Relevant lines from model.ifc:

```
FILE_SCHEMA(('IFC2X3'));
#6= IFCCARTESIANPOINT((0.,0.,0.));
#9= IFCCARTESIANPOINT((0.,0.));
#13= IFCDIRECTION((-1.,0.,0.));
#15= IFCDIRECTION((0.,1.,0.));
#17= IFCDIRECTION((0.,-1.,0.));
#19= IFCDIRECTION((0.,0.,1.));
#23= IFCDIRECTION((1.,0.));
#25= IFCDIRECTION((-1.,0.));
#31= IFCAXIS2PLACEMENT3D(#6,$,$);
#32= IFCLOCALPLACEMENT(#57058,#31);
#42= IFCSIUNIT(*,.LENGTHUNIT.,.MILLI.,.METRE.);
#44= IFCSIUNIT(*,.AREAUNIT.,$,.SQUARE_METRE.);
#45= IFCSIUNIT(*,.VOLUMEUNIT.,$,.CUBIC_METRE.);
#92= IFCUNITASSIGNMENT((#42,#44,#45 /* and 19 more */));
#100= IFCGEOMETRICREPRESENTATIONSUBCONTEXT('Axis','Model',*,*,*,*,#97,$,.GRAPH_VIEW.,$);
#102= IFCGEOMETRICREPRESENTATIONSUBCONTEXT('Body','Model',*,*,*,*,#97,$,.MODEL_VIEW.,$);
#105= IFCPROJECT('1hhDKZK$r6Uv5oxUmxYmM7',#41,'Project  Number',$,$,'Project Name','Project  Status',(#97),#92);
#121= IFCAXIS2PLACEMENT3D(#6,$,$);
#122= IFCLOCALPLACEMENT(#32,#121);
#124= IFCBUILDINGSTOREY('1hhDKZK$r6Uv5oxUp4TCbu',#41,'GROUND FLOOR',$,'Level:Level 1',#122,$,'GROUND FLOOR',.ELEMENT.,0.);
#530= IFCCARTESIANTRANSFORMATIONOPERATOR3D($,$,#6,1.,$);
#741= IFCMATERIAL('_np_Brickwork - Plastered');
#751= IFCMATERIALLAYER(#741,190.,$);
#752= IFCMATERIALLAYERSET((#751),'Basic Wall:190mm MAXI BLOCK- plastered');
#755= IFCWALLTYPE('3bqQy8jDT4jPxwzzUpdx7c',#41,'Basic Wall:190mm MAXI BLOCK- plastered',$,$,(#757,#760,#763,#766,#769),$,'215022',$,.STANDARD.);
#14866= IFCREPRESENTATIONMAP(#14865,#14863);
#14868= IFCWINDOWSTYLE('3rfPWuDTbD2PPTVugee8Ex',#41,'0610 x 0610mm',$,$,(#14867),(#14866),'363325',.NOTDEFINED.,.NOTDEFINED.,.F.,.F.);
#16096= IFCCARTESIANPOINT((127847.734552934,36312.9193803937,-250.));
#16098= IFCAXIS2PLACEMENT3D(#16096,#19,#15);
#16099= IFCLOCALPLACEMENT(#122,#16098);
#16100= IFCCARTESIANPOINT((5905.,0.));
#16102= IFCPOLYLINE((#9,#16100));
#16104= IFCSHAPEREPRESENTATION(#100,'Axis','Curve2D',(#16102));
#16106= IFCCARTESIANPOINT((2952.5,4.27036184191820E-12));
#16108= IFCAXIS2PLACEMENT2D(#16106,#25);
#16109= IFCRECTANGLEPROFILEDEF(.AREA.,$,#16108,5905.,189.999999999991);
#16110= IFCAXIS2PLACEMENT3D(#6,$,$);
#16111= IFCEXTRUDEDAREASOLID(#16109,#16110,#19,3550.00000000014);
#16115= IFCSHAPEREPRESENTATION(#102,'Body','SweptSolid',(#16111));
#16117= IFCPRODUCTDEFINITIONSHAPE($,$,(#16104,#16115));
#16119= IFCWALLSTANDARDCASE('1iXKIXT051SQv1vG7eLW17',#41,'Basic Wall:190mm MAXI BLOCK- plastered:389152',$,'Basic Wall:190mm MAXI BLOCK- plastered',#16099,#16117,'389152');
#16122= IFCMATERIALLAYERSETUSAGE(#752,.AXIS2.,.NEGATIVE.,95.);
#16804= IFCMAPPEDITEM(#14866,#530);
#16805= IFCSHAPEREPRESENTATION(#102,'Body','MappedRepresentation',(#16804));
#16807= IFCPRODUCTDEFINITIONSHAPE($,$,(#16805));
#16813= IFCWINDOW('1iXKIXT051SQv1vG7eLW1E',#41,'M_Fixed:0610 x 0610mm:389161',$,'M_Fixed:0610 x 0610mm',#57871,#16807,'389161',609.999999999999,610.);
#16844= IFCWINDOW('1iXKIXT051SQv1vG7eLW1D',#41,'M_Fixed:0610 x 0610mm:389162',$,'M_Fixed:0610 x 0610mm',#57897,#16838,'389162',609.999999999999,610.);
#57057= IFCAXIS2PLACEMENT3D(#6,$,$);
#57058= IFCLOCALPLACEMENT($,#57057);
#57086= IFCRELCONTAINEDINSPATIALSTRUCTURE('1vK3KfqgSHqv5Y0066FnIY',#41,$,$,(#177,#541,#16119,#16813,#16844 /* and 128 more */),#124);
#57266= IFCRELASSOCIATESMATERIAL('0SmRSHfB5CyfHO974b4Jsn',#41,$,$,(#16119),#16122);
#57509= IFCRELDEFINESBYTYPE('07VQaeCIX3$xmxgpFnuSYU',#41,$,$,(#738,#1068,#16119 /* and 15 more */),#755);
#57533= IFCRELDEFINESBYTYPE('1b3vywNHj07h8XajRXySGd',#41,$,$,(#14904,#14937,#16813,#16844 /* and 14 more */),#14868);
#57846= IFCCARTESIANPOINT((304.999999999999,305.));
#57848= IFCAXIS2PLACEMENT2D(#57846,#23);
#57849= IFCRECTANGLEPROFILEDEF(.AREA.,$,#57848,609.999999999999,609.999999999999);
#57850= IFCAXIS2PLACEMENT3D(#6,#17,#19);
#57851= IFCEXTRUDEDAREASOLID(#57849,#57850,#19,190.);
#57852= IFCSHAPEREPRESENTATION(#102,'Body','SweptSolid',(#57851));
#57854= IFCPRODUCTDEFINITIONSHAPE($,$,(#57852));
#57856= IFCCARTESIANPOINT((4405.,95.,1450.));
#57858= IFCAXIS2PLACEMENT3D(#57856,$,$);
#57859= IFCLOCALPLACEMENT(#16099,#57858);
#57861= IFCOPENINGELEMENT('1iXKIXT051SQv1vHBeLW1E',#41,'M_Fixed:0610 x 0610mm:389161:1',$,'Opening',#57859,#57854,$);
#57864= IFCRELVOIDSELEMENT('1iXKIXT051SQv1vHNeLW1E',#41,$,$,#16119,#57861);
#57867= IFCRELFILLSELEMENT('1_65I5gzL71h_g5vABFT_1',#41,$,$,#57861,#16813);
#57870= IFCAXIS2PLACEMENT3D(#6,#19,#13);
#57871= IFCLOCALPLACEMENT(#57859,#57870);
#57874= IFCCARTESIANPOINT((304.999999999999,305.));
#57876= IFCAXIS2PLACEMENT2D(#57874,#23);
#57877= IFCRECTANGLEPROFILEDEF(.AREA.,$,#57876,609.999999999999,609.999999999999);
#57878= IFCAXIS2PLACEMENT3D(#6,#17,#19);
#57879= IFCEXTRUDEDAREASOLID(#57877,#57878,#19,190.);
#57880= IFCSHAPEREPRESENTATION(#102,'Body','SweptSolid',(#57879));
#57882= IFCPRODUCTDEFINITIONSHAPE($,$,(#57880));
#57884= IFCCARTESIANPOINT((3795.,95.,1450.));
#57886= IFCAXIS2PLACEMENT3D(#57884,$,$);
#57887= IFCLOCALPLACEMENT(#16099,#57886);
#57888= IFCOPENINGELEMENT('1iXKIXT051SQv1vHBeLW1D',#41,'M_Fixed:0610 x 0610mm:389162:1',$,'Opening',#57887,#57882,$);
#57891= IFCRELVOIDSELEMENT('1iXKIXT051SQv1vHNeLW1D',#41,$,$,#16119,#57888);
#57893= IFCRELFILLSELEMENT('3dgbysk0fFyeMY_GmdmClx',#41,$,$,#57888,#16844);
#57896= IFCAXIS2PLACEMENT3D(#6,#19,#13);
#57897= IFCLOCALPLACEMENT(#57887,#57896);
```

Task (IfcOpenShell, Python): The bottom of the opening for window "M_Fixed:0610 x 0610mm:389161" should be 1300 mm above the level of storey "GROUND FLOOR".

```python
import numpy as np
import ifcopenshell
import ifcopenshell.api.geometry
import ifcopenshell.geom
import ifcopenshell.util.element
import ifcopenshell.util.placement
import ifcopenshell.util.shape
import ifcopenshell.util.unit

model = ifcopenshell.open("model.ifc")
unit_scale = ifcopenshell.util.unit.calculate_unit_scale(model)

window = model.by_guid("1iXKIXT051SQv1vG7eLW1E")
opening = window.FillsVoids[0].RelatingOpeningElement
storey = ifcopenshell.util.element.get_container(window, ifc_class="IfcBuildingStorey")
level = ifcopenshell.util.placement.get_local_placement(storey.ObjectPlacement)[2, 3]

# The opening's origin need not be at the sill, so measure its lowest point.
shape = ifcopenshell.geom.create_shape(ifcopenshell.geom.settings(), opening)
bottom = ifcopenshell.util.shape.get_shape_bottom_elevation(shape, shape.geometry) / unit_scale
dz = level + 1300.0 - bottom

shift = np.array([0.0, 0.0, dz])
# The window is placed relative to its opening, so it follows when the opening moves.
matrix = ifcopenshell.util.placement.get_local_placement(opening.ObjectPlacement)
matrix[:3, 3] += shift
ifcopenshell.api.geometry.edit_object_placement(
    model, product=opening, matrix=matrix, is_si=False, should_transform_children=True
)

print(f"moved by {dz * unit_scale:+.3f} m")

model.write("model-out.ifc")
```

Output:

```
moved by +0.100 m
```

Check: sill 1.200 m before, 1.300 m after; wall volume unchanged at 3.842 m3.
